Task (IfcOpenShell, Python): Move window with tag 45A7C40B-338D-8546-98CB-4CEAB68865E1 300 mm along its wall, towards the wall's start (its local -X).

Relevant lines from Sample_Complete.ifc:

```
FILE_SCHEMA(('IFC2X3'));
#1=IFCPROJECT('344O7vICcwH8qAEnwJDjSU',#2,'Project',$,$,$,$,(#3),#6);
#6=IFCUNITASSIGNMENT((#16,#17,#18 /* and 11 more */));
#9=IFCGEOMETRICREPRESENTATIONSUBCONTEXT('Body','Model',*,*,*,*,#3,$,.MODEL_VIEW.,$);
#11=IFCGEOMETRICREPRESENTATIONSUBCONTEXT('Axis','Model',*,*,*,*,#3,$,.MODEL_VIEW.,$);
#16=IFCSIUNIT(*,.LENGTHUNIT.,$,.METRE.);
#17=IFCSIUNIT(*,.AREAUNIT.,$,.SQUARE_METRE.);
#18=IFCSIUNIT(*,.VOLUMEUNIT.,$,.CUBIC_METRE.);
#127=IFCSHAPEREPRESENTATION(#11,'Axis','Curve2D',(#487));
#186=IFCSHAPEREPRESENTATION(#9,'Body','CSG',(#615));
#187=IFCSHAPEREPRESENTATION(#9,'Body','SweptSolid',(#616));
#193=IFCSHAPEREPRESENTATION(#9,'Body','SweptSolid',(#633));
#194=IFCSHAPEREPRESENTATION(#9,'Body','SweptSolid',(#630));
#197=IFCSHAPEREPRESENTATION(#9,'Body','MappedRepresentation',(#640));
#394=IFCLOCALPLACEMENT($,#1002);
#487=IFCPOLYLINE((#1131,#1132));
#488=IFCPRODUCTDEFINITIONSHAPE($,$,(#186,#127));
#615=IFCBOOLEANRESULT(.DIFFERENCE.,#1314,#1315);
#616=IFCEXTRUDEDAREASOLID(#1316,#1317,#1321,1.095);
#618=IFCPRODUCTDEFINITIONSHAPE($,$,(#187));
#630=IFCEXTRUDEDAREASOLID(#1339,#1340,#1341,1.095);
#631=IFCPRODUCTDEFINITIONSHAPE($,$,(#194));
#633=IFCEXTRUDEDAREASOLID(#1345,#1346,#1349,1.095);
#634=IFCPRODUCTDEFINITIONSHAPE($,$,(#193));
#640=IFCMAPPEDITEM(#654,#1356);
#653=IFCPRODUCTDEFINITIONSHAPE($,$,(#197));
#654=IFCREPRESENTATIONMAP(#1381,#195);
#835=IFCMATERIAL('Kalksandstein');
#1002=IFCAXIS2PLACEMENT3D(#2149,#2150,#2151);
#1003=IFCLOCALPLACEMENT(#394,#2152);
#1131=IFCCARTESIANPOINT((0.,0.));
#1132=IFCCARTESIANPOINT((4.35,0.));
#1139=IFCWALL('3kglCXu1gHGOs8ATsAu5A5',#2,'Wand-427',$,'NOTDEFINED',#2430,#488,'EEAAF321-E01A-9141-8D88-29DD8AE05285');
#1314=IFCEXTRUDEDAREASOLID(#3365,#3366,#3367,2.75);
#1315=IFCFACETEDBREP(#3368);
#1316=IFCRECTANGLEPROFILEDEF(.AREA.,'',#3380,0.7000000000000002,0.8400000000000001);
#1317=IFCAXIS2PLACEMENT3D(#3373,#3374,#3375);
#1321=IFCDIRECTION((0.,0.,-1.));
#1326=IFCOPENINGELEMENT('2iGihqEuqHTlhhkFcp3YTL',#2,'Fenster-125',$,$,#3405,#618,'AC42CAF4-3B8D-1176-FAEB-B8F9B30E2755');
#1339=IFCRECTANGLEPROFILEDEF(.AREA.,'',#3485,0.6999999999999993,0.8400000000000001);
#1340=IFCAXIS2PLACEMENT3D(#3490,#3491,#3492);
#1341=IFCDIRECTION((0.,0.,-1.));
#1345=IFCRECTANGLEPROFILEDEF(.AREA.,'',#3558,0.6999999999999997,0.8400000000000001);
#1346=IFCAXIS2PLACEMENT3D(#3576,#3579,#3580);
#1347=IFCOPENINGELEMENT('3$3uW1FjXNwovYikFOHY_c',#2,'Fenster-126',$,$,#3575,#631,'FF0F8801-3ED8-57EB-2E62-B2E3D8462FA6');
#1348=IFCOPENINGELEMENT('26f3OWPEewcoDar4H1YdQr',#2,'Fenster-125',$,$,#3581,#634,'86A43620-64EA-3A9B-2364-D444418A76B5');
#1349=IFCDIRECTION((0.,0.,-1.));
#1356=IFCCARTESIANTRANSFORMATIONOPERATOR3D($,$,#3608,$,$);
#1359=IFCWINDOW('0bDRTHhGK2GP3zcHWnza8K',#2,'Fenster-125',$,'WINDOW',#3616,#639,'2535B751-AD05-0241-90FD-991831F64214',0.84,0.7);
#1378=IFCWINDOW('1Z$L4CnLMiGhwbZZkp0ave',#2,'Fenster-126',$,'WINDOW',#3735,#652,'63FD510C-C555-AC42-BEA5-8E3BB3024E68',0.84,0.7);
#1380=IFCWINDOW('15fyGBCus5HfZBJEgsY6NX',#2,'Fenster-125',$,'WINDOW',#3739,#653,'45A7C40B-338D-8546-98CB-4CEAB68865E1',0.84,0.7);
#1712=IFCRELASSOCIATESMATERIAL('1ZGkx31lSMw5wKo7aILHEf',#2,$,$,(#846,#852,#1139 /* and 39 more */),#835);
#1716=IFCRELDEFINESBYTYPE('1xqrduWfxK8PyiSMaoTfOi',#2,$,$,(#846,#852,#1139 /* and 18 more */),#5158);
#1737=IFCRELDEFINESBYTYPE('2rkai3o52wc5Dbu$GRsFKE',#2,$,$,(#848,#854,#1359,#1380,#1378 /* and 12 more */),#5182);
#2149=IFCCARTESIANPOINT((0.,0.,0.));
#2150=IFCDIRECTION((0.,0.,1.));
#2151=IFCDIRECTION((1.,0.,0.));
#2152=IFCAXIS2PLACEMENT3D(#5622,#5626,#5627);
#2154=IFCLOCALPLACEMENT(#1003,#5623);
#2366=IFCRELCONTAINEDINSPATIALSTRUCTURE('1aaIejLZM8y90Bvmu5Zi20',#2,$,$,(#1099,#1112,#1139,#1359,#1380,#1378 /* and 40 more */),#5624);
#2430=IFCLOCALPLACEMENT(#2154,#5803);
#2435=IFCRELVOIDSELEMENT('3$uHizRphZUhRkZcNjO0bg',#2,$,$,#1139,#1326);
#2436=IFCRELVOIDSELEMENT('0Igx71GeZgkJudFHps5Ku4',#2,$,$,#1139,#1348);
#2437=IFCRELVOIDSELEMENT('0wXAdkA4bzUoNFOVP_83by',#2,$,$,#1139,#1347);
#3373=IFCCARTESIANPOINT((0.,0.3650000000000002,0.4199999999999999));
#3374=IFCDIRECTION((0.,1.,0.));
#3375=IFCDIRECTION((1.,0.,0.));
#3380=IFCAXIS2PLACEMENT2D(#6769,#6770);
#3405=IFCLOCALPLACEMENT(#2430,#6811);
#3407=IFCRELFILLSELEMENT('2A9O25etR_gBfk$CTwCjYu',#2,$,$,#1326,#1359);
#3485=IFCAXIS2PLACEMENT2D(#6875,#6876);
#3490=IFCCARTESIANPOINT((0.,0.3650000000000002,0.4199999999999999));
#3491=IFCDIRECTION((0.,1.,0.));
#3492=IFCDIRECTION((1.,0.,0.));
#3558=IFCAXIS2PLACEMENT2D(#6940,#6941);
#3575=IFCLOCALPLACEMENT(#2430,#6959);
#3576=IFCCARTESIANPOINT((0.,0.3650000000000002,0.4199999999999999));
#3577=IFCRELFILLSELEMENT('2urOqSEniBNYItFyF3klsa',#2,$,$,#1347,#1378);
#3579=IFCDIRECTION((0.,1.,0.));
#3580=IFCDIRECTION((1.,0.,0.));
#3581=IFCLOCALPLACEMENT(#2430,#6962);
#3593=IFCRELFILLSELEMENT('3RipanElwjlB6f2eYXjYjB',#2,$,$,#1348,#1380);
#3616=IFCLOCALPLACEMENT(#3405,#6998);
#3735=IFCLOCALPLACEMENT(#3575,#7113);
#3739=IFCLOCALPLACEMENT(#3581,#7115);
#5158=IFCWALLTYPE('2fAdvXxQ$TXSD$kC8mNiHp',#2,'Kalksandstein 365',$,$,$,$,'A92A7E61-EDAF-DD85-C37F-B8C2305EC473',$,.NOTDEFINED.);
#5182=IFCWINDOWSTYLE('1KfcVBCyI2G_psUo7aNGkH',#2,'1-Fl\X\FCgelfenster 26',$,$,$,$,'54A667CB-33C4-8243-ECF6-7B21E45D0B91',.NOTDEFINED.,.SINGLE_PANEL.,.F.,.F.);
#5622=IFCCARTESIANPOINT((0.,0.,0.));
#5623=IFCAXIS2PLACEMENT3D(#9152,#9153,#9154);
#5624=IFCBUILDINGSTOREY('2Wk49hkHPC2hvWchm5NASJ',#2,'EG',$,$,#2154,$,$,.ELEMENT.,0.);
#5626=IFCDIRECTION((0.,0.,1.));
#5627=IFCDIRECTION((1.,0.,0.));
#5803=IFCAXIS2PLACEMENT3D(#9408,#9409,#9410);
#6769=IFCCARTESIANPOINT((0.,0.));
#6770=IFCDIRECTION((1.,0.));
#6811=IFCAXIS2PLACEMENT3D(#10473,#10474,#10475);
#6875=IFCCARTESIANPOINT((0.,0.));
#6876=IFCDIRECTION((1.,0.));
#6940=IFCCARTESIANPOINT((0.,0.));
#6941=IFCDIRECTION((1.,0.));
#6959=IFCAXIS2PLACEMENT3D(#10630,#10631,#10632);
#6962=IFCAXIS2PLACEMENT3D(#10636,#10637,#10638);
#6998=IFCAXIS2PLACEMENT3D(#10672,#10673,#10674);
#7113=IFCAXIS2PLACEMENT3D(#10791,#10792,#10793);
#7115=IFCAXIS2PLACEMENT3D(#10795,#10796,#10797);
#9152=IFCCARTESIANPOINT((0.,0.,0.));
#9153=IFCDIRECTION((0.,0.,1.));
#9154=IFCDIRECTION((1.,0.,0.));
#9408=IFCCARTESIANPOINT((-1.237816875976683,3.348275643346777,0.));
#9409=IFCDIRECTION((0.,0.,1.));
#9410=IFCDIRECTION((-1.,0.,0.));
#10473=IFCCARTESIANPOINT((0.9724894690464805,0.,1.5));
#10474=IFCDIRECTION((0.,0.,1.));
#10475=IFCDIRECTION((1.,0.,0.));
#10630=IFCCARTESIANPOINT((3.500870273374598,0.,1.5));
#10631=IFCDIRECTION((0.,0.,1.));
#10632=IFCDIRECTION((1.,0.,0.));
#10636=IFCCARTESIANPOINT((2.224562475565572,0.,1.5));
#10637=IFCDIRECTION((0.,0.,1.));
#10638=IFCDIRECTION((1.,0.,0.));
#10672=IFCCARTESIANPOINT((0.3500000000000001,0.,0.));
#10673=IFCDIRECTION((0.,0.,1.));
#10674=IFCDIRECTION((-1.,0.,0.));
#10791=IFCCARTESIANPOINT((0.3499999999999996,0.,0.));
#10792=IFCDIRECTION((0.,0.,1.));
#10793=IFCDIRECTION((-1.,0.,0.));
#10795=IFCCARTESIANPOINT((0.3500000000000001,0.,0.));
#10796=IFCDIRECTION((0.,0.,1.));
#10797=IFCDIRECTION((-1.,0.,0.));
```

```python
import ifcopenshell
import ifcopenshell.api.geometry
import ifcopenshell.util.placement
import ifcopenshell.util.unit

model = ifcopenshell.open("Sample_Complete.ifc")
unit_scale = ifcopenshell.util.unit.calculate_unit_scale(model)

window = model.by_guid("15fyGBCus5HfZBJEgsY6NX")
opening = window.FillsVoids[0].RelatingOpeningElement
wall = opening.VoidsElements[0].RelatingBuildingElement

wall_matrix = ifcopenshell.util.placement.get_local_placement(wall.ObjectPlacement)
shift = wall_matrix[:3, 0] * -0.3 / unit_scale
before = ifcopenshell.util.placement.get_local_placement(window.ObjectPlacement)[:3, 3].copy()

# The window is placed relative to its opening, so it follows when the opening moves.
matrix = ifcopenshell.util.placement.get_local_placement(opening.ObjectPlacement)
matrix[:3, 3] += shift
ifcopenshell.api.geometry.edit_object_placement(
    model, product=opening, matrix=matrix, is_si=False, should_transform_children=True
)

after = ifcopenshell.util.placement.get_local_placement(window.ObjectPlacement)[:3, 3]
print("window moved by", (after - before).round(3) + 0.0)

model.write("Sample_Complete_v2.ifc")
```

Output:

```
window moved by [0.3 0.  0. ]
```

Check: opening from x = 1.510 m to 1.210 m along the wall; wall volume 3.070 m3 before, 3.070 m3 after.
